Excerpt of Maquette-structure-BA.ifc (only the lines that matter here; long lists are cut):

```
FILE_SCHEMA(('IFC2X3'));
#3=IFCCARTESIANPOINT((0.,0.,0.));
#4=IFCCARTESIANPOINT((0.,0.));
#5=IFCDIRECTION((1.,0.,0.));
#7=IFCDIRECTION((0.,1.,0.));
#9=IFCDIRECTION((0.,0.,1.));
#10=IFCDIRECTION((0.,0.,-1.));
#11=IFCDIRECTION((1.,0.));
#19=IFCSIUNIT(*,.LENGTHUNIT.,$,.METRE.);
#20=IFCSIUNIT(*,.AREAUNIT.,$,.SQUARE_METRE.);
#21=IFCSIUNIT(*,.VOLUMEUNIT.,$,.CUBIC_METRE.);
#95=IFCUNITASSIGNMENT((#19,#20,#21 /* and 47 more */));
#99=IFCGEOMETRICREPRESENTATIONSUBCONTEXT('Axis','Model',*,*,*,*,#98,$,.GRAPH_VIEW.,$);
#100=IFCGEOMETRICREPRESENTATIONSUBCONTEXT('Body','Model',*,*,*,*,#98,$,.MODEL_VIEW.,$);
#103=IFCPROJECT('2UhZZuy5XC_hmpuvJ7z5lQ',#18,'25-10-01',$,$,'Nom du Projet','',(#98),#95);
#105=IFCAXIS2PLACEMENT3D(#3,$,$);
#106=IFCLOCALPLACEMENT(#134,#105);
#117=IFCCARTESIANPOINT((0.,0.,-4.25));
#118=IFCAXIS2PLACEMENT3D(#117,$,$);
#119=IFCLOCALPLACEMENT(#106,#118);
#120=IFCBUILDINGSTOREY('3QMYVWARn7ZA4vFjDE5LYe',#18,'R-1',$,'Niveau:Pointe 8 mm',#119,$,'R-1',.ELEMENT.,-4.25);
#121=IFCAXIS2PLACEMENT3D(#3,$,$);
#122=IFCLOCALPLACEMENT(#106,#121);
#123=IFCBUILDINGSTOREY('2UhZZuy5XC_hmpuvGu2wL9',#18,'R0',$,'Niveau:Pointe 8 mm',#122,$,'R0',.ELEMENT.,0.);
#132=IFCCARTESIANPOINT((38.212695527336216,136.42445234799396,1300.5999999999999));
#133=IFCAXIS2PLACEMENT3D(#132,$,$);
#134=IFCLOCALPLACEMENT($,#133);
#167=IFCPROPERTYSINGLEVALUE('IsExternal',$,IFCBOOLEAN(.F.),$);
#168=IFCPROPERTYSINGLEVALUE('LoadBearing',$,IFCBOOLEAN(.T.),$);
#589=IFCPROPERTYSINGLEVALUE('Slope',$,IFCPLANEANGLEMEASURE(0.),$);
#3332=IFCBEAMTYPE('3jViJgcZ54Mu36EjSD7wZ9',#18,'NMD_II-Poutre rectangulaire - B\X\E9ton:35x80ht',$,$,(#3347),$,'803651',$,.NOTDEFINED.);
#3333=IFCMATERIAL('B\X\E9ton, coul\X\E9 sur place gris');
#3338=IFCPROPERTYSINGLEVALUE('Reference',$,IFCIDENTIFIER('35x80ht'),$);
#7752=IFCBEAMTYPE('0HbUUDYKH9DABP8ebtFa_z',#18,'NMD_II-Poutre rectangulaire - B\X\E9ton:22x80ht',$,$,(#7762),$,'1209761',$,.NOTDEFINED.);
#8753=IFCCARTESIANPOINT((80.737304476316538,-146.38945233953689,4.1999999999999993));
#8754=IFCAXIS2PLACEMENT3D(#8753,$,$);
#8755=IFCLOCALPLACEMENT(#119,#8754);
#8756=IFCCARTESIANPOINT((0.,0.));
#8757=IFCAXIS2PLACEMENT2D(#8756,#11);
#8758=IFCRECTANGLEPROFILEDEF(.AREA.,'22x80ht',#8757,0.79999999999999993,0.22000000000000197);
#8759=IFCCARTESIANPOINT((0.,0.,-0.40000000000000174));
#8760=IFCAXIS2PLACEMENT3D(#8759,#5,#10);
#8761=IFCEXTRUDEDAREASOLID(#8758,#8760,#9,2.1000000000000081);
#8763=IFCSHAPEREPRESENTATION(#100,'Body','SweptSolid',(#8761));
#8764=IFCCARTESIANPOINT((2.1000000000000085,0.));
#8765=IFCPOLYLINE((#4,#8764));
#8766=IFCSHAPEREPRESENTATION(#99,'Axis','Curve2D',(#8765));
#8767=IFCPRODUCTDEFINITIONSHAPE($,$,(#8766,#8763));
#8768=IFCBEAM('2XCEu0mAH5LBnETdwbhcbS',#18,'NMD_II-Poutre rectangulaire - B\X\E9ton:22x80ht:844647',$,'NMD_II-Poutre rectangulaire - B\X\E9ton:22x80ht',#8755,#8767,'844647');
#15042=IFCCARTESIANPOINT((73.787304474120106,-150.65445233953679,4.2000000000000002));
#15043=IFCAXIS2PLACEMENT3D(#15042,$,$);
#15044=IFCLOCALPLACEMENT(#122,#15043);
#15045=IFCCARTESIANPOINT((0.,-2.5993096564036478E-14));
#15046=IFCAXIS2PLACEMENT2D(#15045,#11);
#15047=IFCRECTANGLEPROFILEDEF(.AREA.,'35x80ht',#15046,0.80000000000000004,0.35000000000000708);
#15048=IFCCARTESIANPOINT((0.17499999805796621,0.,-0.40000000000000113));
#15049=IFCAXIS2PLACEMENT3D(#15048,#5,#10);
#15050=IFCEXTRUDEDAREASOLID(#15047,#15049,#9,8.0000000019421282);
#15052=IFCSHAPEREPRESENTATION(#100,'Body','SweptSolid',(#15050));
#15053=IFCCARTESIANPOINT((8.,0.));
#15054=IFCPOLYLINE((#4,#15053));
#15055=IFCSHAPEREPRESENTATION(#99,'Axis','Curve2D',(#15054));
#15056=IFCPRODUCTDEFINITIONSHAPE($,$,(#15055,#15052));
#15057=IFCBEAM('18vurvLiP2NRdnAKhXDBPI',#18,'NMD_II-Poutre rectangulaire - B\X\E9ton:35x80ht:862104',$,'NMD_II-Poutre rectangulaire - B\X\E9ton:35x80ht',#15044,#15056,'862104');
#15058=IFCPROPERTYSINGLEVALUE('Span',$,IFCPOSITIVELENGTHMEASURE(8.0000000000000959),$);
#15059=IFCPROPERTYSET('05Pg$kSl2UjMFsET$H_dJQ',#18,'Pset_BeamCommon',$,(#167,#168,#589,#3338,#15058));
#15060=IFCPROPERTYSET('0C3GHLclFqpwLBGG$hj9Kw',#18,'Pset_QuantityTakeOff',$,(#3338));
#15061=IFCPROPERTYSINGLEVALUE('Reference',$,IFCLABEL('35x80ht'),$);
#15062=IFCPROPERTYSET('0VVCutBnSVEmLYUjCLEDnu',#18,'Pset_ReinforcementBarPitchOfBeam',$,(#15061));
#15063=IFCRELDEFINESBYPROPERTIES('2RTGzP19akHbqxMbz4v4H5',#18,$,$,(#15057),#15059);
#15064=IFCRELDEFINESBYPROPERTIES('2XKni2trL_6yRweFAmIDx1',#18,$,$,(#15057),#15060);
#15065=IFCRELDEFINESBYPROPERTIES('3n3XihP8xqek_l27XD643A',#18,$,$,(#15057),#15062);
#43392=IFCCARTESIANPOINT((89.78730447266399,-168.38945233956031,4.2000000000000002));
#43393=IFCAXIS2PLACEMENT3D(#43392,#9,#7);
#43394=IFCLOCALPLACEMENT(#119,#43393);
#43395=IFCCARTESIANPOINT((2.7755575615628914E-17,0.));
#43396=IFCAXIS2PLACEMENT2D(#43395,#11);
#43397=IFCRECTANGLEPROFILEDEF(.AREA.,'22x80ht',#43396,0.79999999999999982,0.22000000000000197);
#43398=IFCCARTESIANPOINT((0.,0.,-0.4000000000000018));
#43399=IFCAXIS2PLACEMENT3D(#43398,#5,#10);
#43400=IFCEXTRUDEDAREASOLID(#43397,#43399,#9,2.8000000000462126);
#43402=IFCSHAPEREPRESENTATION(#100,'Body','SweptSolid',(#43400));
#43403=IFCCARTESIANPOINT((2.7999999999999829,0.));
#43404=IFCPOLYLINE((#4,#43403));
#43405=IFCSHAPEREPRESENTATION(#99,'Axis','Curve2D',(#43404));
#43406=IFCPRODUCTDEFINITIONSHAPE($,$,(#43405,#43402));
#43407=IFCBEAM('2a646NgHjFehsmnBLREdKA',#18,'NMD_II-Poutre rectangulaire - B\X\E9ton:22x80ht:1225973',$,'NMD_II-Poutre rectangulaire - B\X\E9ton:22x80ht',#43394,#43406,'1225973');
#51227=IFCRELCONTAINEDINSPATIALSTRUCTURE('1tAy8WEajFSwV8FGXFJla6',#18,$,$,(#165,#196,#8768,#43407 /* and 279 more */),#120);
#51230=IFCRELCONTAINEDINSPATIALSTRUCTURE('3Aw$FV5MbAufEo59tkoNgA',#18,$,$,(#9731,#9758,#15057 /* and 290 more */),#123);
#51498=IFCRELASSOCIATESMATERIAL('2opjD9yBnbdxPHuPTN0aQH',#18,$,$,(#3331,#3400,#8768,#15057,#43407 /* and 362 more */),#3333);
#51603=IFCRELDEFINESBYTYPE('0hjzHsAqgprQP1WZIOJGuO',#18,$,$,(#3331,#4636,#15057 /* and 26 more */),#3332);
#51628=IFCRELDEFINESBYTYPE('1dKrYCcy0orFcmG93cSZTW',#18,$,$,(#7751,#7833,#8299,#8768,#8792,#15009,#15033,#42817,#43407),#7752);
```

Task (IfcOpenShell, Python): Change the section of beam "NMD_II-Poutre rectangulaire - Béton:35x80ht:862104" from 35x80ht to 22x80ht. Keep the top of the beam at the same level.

```python
import ifcopenshell
import ifcopenshell.api.pset
import ifcopenshell.api.type
import ifcopenshell.util.element
import ifcopenshell.util.representation

model = ifcopenshell.open("Maquette-structure-BA.ifc")

member = model.by_guid("18vurvLiP2NRdnAKhXDBPI")
source = next(p for p in model.by_type("IfcRectangleProfileDef") if p.ProfileName == "22x80ht")

body = ifcopenshell.util.representation.get_representation(member, "Model", "Body")
solid = body.Items[0]
old_profile = solid.SweptArea

# Copy the section's sizes but keep this member's own profile position.
profile = ifcopenshell.util.element.copy(model, source)
# Profiles are centred, so shift by half the change in depth to hold the top.
shift = (old_profile.XDim - profile.XDim) / 2
x, y = old_profile.Position.Location.Coordinates
up = (-1.0, 0.0)  # upwards, in the solid's own plane
location = model.createIfcCartesianPoint((x + up[0] * shift, y + up[1] * shift))
profile.Position = model.createIfcAxis2Placement2D(location, old_profile.Position.RefDirection)
solid.SweptArea = profile
if not model.get_total_inverses(old_profile):
    ifcopenshell.util.element.remove_deep2(model, old_profile)

new_type = model.by_guid("0HbUUDYKH9DABP8ebtFa_z")
ifcopenshell.api.type.assign_type(
    model, related_objects=[member], relating_type=new_type, should_map_representations=False
)
member.Name = member.Name.replace("35x80ht", "22x80ht")
member.ObjectType = "NMD_II-Poutre rectangulaire - Béton:22x80ht"
pset = model.by_id(ifcopenshell.util.element.get_pset(member, "Pset_BeamCommon", should_inherit=False)["id"])
ifcopenshell.api.pset.edit_pset(model, pset=pset, properties={"Reference": "22x80ht"})
pset = model.by_id(ifcopenshell.util.element.get_pset(member, "Pset_QuantityTakeOff", should_inherit=False)["id"])
ifcopenshell.api.pset.edit_pset(model, pset=pset, properties={"Reference": "22x80ht"})
pset = model.by_id(ifcopenshell.util.element.get_pset(member, "Pset_ReinforcementBarPitchOfBeam", should_inherit=False)["id"])
ifcopenshell.api.pset.edit_pset(model, pset=pset, properties={"Reference": "22x80ht"})

print(solid.SweptArea)

model.write("Maquette-structure-BA_updated.ifc")
```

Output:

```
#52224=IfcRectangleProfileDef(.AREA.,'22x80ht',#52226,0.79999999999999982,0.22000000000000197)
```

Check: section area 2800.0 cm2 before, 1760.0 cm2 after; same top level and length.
